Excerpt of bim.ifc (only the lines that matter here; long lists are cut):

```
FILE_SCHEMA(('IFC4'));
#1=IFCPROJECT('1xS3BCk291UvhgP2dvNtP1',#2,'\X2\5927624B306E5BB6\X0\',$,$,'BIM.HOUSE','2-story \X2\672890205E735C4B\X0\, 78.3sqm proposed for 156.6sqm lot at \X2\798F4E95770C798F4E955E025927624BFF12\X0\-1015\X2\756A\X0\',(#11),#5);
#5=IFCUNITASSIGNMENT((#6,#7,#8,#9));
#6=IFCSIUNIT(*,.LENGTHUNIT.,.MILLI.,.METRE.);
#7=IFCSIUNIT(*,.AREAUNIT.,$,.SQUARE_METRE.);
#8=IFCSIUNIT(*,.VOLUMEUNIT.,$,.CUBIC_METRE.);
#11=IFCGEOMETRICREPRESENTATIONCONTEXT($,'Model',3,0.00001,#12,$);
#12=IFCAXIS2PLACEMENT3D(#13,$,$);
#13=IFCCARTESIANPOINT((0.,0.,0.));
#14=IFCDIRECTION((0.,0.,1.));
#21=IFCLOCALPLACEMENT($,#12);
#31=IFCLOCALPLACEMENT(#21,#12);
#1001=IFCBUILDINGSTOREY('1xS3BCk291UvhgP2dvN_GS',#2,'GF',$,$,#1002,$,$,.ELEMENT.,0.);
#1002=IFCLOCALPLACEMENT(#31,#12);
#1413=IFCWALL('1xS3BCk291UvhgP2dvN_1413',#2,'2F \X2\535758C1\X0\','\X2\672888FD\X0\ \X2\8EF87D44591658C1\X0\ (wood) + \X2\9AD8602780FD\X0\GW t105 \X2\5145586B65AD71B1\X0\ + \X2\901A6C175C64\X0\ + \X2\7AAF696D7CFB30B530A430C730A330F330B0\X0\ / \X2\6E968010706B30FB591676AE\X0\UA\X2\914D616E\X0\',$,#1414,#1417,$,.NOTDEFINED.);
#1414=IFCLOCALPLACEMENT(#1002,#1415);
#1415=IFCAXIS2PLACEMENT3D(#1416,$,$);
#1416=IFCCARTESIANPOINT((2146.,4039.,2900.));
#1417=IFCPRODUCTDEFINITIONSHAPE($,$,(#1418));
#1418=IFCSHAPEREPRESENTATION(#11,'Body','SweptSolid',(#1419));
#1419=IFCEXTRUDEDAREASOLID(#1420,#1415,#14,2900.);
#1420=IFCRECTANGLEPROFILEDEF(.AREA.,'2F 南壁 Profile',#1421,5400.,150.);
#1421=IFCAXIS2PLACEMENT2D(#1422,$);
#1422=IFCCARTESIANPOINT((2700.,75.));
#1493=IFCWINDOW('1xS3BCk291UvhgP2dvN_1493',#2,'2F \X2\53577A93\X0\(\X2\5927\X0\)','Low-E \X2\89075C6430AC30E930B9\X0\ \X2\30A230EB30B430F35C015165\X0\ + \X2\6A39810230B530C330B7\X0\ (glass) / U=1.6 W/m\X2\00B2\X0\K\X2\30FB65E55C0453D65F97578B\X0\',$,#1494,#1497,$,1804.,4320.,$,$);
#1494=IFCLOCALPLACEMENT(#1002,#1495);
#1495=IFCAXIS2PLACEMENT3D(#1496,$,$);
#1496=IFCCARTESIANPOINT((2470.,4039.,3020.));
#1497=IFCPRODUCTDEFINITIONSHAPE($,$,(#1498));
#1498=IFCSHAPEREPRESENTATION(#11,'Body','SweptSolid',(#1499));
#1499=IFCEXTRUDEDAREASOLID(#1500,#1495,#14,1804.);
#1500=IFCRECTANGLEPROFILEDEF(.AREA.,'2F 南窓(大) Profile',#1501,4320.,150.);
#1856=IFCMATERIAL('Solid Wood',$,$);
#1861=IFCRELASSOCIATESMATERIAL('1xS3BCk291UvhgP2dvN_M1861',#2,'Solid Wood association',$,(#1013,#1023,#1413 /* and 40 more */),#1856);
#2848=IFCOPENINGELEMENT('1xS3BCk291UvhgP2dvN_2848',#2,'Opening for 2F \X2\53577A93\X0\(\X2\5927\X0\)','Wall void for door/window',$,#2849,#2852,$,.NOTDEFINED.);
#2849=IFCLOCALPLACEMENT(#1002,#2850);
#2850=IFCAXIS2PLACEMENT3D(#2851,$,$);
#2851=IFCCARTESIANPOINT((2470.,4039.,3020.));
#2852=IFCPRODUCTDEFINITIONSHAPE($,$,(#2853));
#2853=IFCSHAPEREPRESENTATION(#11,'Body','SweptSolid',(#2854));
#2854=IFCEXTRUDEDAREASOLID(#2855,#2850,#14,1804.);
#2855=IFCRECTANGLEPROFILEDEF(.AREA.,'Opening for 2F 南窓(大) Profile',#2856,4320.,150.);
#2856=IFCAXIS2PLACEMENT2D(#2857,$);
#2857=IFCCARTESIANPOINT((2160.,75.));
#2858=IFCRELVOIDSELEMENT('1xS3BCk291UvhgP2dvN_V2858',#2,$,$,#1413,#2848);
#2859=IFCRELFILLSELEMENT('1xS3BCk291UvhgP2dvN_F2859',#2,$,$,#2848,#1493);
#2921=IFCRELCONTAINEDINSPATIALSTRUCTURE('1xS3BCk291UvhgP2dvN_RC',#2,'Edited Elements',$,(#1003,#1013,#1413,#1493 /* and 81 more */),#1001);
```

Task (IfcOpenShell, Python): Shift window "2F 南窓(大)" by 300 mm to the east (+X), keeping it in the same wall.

```python
import ifcopenshell
import ifcopenshell.api.geometry
import ifcopenshell.util.placement
import ifcopenshell.util.unit

model = ifcopenshell.open("bim.ifc")
unit_scale = ifcopenshell.util.unit.calculate_unit_scale(model)

window = model.by_guid("1xS3BCk291UvhgP2dvN_1493")
opening = window.FillsVoids[0].RelatingOpeningElement
wall = opening.VoidsElements[0].RelatingBuildingElement

wall_matrix = ifcopenshell.util.placement.get_local_placement(wall.ObjectPlacement)
shift = wall_matrix[:3, 0] * 0.3 / unit_scale
before = ifcopenshell.util.placement.get_local_placement(window.ObjectPlacement)[:3, 3].copy()

# The window is not placed relative to its opening, so move both.
for product in (opening, window):
    matrix = ifcopenshell.util.placement.get_local_placement(product.ObjectPlacement)
    matrix[:3, 3] += shift
    ifcopenshell.api.geometry.edit_object_placement(model, product=product, matrix=matrix, is_si=False)

after = ifcopenshell.util.placement.get_local_placement(window.ObjectPlacement)[:3, 3]
print("window moved by", (after - before).round(3) + 0.0)

model.write("bim_edited.ifc")
```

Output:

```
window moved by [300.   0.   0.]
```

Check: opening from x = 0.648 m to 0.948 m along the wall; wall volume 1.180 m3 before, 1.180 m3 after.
